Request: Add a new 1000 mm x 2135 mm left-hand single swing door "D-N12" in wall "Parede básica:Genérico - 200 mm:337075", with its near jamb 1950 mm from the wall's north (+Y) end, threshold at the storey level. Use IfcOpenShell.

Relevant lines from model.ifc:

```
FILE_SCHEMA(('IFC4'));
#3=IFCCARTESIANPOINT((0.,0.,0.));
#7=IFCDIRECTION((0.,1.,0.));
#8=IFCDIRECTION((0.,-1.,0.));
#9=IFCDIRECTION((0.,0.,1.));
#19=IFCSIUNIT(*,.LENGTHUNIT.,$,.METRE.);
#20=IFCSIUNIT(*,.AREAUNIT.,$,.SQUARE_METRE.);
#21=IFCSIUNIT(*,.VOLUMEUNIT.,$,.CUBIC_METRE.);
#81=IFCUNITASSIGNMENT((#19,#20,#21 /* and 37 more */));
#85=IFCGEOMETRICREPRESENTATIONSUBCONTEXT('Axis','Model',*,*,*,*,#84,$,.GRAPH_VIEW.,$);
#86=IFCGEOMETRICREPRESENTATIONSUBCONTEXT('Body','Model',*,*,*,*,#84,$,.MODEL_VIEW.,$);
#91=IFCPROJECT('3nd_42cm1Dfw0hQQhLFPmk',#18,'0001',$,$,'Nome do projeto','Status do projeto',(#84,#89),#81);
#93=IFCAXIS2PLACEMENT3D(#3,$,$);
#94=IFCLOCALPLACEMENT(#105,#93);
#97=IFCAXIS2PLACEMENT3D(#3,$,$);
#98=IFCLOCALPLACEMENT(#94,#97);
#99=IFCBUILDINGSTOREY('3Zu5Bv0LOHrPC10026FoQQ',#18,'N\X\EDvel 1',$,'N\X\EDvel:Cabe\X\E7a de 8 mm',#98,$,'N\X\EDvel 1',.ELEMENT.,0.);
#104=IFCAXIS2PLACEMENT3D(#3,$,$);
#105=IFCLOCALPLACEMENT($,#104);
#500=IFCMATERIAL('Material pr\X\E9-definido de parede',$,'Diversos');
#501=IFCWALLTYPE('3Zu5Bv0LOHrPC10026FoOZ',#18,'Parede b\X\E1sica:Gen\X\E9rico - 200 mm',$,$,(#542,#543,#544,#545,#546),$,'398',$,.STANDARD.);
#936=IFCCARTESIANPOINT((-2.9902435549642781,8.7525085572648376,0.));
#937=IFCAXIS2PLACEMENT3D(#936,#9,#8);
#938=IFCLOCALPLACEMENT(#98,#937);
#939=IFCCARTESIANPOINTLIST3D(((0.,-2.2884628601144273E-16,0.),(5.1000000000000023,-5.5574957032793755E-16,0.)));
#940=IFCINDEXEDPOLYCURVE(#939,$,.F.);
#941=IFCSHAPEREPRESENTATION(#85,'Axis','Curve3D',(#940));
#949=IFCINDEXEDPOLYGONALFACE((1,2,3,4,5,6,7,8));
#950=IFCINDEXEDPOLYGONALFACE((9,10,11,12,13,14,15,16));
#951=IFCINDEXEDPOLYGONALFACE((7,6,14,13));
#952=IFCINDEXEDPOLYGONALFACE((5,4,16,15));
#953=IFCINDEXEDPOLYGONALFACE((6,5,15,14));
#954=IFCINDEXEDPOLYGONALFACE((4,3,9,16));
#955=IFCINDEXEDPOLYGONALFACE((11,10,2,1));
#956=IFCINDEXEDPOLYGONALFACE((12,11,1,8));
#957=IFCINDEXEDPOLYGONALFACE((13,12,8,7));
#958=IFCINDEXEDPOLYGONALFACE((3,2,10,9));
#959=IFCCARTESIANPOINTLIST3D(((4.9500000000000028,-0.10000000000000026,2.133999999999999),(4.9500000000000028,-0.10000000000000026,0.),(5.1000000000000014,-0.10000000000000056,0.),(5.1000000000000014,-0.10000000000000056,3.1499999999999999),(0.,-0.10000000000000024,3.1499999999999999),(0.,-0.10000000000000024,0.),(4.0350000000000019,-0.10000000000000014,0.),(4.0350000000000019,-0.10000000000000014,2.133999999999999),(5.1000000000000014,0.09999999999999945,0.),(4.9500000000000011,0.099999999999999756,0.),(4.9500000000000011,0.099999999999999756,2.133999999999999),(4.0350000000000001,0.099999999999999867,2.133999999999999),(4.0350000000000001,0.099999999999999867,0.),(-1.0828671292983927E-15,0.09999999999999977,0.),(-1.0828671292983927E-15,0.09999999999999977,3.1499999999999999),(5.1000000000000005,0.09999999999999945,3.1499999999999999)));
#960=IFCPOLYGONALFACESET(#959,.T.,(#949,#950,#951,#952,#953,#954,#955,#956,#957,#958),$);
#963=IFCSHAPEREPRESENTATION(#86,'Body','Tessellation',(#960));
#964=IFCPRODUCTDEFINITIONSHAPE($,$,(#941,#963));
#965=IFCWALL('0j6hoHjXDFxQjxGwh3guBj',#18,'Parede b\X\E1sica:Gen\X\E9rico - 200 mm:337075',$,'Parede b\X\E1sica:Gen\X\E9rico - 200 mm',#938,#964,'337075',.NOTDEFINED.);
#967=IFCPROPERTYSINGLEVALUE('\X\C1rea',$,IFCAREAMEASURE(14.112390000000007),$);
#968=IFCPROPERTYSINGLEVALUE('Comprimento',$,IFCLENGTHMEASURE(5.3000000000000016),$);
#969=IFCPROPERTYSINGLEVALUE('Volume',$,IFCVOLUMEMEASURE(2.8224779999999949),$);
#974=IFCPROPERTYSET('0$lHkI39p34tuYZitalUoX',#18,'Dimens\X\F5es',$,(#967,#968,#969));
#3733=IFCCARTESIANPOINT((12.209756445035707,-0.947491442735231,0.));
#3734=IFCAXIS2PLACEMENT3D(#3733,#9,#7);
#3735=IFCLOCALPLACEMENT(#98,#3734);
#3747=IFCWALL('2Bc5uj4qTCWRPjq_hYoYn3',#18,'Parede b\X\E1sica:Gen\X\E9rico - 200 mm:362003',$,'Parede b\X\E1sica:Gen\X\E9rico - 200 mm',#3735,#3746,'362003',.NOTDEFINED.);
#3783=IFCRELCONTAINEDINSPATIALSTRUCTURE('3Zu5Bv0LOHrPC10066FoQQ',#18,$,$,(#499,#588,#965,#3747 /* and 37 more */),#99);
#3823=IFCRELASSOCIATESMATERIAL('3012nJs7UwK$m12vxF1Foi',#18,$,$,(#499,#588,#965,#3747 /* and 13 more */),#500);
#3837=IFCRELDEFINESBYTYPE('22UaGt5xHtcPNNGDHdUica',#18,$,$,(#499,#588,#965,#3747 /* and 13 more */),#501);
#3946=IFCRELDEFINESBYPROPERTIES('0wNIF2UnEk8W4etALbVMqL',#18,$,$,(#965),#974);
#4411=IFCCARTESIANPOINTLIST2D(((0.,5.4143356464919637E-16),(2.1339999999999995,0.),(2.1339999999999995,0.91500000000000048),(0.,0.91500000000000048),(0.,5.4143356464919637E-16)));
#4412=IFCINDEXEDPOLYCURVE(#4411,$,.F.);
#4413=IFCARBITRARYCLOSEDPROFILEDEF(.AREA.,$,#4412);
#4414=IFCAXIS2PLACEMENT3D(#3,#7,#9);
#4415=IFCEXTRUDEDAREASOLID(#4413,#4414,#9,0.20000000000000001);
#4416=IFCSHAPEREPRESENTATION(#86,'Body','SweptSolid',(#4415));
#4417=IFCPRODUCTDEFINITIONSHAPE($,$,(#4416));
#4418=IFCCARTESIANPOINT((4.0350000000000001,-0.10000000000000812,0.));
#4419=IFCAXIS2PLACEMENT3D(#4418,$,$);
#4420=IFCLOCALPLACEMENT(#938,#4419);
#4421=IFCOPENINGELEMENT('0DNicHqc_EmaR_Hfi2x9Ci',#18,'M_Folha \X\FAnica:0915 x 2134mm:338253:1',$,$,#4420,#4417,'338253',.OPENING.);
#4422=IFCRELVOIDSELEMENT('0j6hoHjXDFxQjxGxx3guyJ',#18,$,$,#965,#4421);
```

```python
import numpy as np
import ifcopenshell
import ifcopenshell.api.feature
import ifcopenshell.api.geometry
import ifcopenshell.api.pset
import ifcopenshell.api.root
import ifcopenshell.api.spatial
import ifcopenshell.geom
import ifcopenshell.util.element
import ifcopenshell.util.placement
import ifcopenshell.util.representation
import ifcopenshell.util.shape
import ifcopenshell.util.unit

model = ifcopenshell.open("model.ifc")
unit_scale = ifcopenshell.util.unit.calculate_unit_scale(model)
area_scale = ifcopenshell.util.unit.calculate_unit_scale(model, "AREAUNIT")
volume_scale = ifcopenshell.util.unit.calculate_unit_scale(model, "VOLUMEUNIT")
settings = ifcopenshell.geom.settings()


def volume(element):
    """Net volume in cubic metres, openings subtracted."""
    shape = ifcopenshell.geom.create_shape(settings, element)
    return ifcopenshell.util.shape.get_volume(shape.geometry)


wall = model.by_guid("0j6hoHjXDFxQjxGwh3guBj")
storey = ifcopenshell.util.element.get_container(wall, ifc_class="IfcBuildingStorey")
context = ifcopenshell.util.representation.get_context(model, "Model", "Body", "MODEL_VIEW")
before = volume(wall)

width, height, from_end, sill = 1, 2.135, 1.95, 0.0  # metres

# The wall runs along its own X axis, and the end named is its -X end.
wall_shape = ifcopenshell.geom.create_shape(settings, wall)
x, y, z = ifcopenshell.util.shape.get_vertices(wall_shape.geometry).T
start = x.min() + from_end
face, thickness = float(y.min()), float(y.max() - y.min())
wall_matrix = ifcopenshell.util.placement.get_local_placement(wall.ObjectPlacement)
level = ifcopenshell.util.placement.get_local_placement(storey.ObjectPlacement)[2, 3]


def in_wall(x, y):
    """Placement at x, y metres in the wall's axes, at sill height."""
    matrix = wall_matrix.copy()
    matrix[:, 3] = wall_matrix @ np.array([x / unit_scale, y / unit_scale, 0.0, 1.0])
    matrix[2, 3] = level + sill / unit_scale
    return matrix


# Opening: a box that overshoots both wall faces by 50 mm.
opening = ifcopenshell.api.root.create_entity(model, ifc_class="IfcOpeningElement", predefined_type="OPENING")
box = ifcopenshell.api.geometry.add_wall_representation(
    model, context=context, length=width, height=height, thickness=thickness + 0.1
)
ifcopenshell.api.geometry.assign_representation(model, product=opening, representation=box)
ifcopenshell.api.geometry.edit_object_placement(model, product=opening, matrix=in_wall(start, face - 0.05), is_si=False)
ifcopenshell.api.feature.add_feature(model, feature=opening, element=wall)

door = ifcopenshell.api.root.create_entity(model, ifc_class="IfcDoor", name="D-N12", predefined_type="DOOR")
door.OverallWidth, door.OverallHeight = width / unit_scale, height / unit_scale
door.OperationType = "SINGLE_SWING_LEFT"
body = ifcopenshell.api.geometry.add_door_representation(
    model,
    context=context,
    overall_width=door.OverallWidth,
    overall_height=door.OverallHeight,
    operation_type="SINGLE_SWING_LEFT",
    lining_properties={"LiningDepth": thickness / unit_scale, "ThresholdDepth": thickness / unit_scale},
)
ifcopenshell.api.geometry.assign_representation(model, product=door, representation=body)
ifcopenshell.api.spatial.assign_container(model, products=[door], relating_structure=storey)
ifcopenshell.api.feature.add_filling(model, opening=opening, element=door)

# The lining spans the wall, so the door starts at the wall face.
ifcopenshell.api.geometry.edit_object_placement(model, product=door, matrix=in_wall(start, face), is_si=False)

after = volume(wall)

# Update the wall's stored quantities.
pset = model.by_id(ifcopenshell.util.element.get_pset(wall, "Dimensões", should_inherit=False)["id"])
ifcopenshell.api.pset.edit_pset(model, pset=pset, properties={
    "Área": model.create_entity("IfcAreaMeasure", after / thickness / area_scale),
    "Volume": model.create_entity("IfcVolumeMeasure", after / volume_scale),
})

print(f"wall volume {before:.3f} -> {after:.3f} m3")

model.write("model_rev.ifc")
```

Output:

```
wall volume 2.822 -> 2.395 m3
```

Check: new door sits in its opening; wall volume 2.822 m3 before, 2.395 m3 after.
